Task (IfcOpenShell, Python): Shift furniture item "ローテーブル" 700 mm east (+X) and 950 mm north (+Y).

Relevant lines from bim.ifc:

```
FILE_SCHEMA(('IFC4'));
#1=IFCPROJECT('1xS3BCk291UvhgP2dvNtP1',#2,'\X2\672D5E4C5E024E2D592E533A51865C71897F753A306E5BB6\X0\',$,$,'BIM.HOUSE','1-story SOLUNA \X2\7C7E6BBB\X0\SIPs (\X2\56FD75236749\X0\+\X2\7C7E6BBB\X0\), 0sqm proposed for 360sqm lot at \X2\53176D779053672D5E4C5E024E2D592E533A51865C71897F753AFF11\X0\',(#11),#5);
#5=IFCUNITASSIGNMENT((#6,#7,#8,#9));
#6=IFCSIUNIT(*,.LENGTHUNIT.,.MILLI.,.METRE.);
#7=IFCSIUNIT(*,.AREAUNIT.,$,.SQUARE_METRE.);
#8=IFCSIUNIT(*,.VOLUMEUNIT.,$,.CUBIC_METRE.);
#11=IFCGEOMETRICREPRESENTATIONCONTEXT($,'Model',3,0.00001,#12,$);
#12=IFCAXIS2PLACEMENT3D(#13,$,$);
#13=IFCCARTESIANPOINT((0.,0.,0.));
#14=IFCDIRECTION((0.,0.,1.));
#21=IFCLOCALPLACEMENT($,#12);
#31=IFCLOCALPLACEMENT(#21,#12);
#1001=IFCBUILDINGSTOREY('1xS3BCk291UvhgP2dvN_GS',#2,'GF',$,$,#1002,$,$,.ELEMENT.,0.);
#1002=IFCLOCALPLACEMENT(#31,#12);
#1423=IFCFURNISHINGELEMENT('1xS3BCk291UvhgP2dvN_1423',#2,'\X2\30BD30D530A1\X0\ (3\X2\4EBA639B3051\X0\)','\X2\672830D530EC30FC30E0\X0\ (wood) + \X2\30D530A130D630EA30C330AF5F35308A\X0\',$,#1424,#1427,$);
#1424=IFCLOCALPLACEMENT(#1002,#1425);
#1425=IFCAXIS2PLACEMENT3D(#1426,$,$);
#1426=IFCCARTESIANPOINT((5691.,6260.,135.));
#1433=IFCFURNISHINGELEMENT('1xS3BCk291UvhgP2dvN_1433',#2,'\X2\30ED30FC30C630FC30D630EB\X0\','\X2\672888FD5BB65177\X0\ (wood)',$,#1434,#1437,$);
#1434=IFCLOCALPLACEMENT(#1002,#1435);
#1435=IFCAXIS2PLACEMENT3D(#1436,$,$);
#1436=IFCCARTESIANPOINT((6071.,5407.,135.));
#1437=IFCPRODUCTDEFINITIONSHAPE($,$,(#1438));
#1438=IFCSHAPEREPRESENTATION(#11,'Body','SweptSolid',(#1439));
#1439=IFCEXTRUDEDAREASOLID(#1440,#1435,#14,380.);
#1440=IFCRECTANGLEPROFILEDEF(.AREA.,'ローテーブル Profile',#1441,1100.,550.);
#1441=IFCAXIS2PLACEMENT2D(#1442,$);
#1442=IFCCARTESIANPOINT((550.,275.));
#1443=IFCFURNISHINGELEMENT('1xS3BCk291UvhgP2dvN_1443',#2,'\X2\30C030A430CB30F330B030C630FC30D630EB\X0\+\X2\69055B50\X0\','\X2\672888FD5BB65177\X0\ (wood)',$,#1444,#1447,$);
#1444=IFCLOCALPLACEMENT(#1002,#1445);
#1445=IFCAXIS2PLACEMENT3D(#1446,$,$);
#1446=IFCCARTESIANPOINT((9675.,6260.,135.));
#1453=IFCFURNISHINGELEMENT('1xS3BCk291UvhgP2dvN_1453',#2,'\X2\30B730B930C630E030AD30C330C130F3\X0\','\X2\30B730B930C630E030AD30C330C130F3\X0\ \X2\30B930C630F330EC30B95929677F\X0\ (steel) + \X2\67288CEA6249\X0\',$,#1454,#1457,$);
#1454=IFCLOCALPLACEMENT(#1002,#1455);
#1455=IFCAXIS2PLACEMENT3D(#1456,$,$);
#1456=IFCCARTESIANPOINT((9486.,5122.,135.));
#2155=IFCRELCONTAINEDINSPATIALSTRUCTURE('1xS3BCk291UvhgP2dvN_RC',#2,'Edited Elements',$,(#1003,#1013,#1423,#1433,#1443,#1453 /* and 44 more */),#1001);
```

```python
import ifcopenshell
import ifcopenshell.api.geometry
import ifcopenshell.util.placement

model = ifcopenshell.open("bim.ifc")

item = model.by_guid("1xS3BCk291UvhgP2dvN_1433")
matrix = ifcopenshell.util.placement.get_local_placement(item.ObjectPlacement)
matrix[0, 3] += 700.0
matrix[1, 3] += 950.0
ifcopenshell.api.geometry.edit_object_placement(model, product=item, matrix=matrix, is_si=False)

print(ifcopenshell.util.placement.get_local_placement(item.ObjectPlacement).round(3) + 0.0)

model.write("bim_updated.ifc")
```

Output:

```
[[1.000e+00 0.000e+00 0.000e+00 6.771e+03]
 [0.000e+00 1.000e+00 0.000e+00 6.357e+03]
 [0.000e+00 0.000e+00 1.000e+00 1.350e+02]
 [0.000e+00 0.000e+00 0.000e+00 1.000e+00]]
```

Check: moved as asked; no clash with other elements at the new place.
